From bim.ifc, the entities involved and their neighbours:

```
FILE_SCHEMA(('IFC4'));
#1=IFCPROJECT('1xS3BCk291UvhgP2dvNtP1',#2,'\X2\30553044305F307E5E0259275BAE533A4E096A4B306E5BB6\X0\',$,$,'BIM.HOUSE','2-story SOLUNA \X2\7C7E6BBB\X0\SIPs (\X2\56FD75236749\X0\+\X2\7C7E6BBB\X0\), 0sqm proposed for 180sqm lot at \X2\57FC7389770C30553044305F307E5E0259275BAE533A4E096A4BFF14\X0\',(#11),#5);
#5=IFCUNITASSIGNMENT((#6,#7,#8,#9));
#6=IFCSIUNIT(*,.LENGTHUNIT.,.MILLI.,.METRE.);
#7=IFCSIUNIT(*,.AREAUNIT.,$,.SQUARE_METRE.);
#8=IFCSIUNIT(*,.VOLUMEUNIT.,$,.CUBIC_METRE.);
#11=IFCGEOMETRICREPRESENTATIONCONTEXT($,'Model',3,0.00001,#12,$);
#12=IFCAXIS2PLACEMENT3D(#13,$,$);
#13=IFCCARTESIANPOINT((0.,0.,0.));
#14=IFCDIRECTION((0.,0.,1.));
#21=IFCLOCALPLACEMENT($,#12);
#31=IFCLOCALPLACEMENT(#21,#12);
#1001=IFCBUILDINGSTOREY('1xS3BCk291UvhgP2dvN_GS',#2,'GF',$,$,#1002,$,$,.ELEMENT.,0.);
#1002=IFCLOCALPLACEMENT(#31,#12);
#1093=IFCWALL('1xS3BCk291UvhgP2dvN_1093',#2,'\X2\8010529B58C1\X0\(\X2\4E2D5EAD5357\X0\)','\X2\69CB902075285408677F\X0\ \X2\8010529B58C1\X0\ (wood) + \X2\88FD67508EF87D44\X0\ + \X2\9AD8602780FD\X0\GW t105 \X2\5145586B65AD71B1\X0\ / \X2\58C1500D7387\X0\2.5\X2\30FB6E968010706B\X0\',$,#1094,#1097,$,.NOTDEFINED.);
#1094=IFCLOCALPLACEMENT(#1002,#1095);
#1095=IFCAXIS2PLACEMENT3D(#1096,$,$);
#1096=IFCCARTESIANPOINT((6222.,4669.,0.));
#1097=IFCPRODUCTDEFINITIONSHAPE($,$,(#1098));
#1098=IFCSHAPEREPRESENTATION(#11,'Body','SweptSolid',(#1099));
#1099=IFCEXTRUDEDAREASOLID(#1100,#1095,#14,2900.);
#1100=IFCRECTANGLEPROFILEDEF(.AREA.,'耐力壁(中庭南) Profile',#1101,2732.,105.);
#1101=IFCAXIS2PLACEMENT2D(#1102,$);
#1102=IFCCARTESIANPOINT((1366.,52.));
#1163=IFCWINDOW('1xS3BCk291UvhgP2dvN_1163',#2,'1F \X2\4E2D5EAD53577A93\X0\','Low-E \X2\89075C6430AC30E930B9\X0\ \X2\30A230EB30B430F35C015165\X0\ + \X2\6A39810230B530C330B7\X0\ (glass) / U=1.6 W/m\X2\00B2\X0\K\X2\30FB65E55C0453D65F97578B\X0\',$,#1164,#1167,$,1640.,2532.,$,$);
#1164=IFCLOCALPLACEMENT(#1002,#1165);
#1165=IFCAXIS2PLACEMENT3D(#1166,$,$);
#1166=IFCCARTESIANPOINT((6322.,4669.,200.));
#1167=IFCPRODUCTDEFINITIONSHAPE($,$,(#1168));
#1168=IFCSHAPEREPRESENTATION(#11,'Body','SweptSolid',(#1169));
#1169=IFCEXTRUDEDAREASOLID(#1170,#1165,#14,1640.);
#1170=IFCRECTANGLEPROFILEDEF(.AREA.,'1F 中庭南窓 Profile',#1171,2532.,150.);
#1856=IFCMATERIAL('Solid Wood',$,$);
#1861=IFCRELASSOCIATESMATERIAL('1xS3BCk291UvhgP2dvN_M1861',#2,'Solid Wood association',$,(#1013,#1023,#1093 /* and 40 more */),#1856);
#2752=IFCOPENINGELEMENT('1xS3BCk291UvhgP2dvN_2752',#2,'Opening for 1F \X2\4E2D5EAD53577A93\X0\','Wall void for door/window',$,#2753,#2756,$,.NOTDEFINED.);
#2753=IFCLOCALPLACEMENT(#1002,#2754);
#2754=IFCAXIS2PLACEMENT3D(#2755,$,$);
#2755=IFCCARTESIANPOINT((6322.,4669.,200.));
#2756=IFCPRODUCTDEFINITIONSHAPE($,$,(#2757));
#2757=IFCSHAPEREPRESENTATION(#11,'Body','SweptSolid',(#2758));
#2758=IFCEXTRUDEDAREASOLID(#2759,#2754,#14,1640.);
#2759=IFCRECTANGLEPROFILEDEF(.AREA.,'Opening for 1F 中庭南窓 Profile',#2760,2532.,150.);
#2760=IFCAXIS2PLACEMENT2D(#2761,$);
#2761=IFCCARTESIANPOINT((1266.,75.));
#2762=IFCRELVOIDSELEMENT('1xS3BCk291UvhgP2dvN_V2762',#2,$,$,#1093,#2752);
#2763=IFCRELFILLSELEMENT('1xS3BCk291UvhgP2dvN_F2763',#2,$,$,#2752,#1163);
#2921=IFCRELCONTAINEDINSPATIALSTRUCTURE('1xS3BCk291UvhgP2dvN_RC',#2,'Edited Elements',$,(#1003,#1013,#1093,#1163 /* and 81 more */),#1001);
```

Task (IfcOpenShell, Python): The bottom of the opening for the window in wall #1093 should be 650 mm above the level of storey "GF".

```python
import numpy as np
import ifcopenshell
import ifcopenshell.api.geometry
import ifcopenshell.geom
import ifcopenshell.util.element
import ifcopenshell.util.placement
import ifcopenshell.util.shape
import ifcopenshell.util.unit

model = ifcopenshell.open("bim.ifc")
unit_scale = ifcopenshell.util.unit.calculate_unit_scale(model)

window = model.by_id(1163)
opening = window.FillsVoids[0].RelatingOpeningElement
storey = ifcopenshell.util.element.get_container(window, ifc_class="IfcBuildingStorey")
level = ifcopenshell.util.placement.get_local_placement(storey.ObjectPlacement)[2, 3]

# The opening's origin need not be at the sill, so measure its lowest point.
shape = ifcopenshell.geom.create_shape(ifcopenshell.geom.settings(), opening)
bottom = ifcopenshell.util.shape.get_shape_bottom_elevation(shape, shape.geometry) / unit_scale
dz = level + 650.0 - bottom

shift = np.array([0.0, 0.0, dz])
# The window is not placed relative to its opening, so move both.
for product in (opening, window):
    matrix = ifcopenshell.util.placement.get_local_placement(product.ObjectPlacement)
    matrix[:3, 3] += shift
    ifcopenshell.api.geometry.edit_object_placement(model, product=product, matrix=matrix, is_si=False)

print(f"moved by {dz * unit_scale:+.3f} m")

model.write("bim_edited.ifc")
```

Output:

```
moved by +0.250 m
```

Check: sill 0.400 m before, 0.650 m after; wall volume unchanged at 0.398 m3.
